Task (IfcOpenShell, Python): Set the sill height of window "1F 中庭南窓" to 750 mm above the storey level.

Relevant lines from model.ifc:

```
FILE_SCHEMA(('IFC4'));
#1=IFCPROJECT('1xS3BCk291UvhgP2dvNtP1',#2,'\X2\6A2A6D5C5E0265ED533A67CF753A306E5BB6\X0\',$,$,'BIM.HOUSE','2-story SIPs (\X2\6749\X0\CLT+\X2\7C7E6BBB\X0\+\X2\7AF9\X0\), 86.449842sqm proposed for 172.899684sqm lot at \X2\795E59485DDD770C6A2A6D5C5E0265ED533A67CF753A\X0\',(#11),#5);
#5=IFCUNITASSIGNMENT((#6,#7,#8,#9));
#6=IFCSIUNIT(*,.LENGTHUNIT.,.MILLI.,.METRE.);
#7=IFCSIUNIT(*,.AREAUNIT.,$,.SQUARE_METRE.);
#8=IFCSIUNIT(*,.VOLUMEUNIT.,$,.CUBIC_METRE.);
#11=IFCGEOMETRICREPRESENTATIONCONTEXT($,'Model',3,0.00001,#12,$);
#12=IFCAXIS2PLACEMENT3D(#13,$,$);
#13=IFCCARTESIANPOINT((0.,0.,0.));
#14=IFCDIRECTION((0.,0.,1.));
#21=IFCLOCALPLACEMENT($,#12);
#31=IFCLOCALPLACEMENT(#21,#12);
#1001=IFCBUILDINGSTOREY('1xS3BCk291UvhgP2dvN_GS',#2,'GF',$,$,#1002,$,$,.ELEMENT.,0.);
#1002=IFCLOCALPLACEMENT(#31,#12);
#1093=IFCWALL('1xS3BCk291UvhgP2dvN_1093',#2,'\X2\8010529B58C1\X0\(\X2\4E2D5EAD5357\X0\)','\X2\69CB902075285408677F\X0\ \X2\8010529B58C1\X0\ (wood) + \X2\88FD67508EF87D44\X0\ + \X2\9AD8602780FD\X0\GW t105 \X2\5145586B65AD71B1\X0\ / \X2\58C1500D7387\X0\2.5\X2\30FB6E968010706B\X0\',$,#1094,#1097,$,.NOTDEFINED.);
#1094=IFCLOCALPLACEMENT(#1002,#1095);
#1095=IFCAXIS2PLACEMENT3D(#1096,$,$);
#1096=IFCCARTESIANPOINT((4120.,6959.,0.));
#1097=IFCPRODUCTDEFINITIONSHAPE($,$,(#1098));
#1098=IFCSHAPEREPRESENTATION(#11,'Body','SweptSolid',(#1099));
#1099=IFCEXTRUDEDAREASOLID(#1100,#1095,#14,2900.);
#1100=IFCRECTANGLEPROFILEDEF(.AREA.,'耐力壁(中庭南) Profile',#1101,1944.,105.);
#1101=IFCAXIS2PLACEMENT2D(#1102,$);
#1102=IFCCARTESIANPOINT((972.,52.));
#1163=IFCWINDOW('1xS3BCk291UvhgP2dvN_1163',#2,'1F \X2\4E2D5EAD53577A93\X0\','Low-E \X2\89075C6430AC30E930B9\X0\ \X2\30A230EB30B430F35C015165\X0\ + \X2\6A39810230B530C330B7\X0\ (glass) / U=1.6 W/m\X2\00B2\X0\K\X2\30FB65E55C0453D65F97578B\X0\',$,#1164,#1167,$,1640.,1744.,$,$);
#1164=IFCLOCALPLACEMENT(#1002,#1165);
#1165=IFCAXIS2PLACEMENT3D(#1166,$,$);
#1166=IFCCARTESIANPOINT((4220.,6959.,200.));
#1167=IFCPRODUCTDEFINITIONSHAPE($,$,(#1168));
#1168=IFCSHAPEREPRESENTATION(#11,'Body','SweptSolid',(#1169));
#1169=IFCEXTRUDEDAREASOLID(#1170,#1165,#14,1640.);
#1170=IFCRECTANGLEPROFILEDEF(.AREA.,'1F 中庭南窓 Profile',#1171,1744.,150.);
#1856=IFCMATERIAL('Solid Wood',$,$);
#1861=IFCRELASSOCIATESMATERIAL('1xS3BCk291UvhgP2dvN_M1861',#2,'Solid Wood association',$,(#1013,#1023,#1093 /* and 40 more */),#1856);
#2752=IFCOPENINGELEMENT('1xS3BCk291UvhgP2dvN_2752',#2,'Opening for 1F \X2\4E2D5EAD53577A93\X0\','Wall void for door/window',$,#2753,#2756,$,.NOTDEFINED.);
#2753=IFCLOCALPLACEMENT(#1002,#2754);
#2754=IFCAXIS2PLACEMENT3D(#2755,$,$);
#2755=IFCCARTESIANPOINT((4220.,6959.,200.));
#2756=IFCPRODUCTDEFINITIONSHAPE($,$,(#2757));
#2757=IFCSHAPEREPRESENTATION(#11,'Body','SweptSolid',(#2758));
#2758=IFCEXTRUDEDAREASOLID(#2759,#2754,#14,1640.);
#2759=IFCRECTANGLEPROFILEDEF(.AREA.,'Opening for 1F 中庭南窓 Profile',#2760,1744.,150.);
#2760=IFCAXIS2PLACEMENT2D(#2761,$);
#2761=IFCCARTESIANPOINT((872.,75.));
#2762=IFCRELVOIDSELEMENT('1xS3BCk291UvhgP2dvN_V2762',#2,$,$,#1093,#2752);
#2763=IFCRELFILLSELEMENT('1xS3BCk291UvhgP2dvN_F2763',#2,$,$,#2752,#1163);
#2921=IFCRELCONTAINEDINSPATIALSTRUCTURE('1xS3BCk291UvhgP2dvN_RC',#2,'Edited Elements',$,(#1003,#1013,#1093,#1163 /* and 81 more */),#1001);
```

```python
import numpy as np
import ifcopenshell
import ifcopenshell.api.geometry
import ifcopenshell.geom
import ifcopenshell.util.element
import ifcopenshell.util.placement
import ifcopenshell.util.shape
import ifcopenshell.util.unit

model = ifcopenshell.open("model.ifc")
unit_scale = ifcopenshell.util.unit.calculate_unit_scale(model)

window = model.by_id(1163)
opening = window.FillsVoids[0].RelatingOpeningElement
storey = ifcopenshell.util.element.get_container(window, ifc_class="IfcBuildingStorey")
level = ifcopenshell.util.placement.get_local_placement(storey.ObjectPlacement)[2, 3]

# The opening's origin need not be at the sill, so measure its lowest point.
shape = ifcopenshell.geom.create_shape(ifcopenshell.geom.settings(), opening)
bottom = ifcopenshell.util.shape.get_shape_bottom_elevation(shape, shape.geometry) / unit_scale
dz = level + 750.0 - bottom

shift = np.array([0.0, 0.0, dz])
# The window is not placed relative to its opening, so move both.
for product in (opening, window):
    matrix = ifcopenshell.util.placement.get_local_placement(product.ObjectPlacement)
    matrix[:3, 3] += shift
    ifcopenshell.api.geometry.edit_object_placement(model, product=product, matrix=matrix, is_si=False)

print(f"moved by {dz * unit_scale:+.3f} m")

model.write("model_rev.ifc")
```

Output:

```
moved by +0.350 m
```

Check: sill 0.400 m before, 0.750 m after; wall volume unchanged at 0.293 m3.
